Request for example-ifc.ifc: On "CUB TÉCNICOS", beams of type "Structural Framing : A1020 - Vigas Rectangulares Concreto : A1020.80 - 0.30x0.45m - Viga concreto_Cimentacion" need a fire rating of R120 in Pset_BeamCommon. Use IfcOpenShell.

First a look at what the model holds.

```python
import ifcopenshell
import ifcopenshell.util.element

model = ifcopenshell.open("example-ifc.ifc")
print(model.schema)
storey = next(s for s in model.by_type("IfcBuildingStorey") if s.Name == "CUB TÉCNICOS")
beams = [e for e in ifcopenshell.util.element.get_decomposition(storey) if e.is_a("IfcBeam")]
seen = {}
for e in beams:
    element_type = ifcopenshell.util.element.get_type(e)
    key = (element_type.Name if element_type != e and element_type else None, ifcopenshell.util.element.get_pset(e, "Pset_BeamCommon", "FireRating"))
    seen[key] = seen.get(key, 0) + 1
for (name, value), count in sorted(seen.items(), key=str):
    print(count, "x", name, "|", value)
```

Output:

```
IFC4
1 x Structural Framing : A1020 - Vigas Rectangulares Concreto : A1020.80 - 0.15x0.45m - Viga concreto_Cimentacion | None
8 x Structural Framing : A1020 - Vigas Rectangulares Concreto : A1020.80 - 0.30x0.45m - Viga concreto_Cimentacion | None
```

```python
import ifcopenshell
import ifcopenshell.api.pset
import ifcopenshell.util.element

model = ifcopenshell.open("example-ifc.ifc")

storey = next(s for s in model.by_type("IfcBuildingStorey") if s.Name == "CUB TÉCNICOS")
beams = [e for e in ifcopenshell.util.element.get_decomposition(storey) if e.is_a("IfcBeam")]

count = 0
for e in beams:
    element_type = ifcopenshell.util.element.get_type(e)
    if element_type in (None, e) or element_type.Name != "Structural Framing : A1020 - Vigas Rectangulares Concreto : A1020.80 - 0.30x0.45m - Viga concreto_Cimentacion":
        continue
    # add_pset returns the element's existing set when there is one.
    pset = ifcopenshell.api.pset.add_pset(model, product=e, name="Pset_BeamCommon")
    ifcopenshell.api.pset.edit_pset(model, pset=pset, properties={"FireRating": "R120"})
    count += 1

print(count, "beams updated")

model.write("example-ifc-out.ifc")
```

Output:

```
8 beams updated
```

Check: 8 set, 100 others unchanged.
